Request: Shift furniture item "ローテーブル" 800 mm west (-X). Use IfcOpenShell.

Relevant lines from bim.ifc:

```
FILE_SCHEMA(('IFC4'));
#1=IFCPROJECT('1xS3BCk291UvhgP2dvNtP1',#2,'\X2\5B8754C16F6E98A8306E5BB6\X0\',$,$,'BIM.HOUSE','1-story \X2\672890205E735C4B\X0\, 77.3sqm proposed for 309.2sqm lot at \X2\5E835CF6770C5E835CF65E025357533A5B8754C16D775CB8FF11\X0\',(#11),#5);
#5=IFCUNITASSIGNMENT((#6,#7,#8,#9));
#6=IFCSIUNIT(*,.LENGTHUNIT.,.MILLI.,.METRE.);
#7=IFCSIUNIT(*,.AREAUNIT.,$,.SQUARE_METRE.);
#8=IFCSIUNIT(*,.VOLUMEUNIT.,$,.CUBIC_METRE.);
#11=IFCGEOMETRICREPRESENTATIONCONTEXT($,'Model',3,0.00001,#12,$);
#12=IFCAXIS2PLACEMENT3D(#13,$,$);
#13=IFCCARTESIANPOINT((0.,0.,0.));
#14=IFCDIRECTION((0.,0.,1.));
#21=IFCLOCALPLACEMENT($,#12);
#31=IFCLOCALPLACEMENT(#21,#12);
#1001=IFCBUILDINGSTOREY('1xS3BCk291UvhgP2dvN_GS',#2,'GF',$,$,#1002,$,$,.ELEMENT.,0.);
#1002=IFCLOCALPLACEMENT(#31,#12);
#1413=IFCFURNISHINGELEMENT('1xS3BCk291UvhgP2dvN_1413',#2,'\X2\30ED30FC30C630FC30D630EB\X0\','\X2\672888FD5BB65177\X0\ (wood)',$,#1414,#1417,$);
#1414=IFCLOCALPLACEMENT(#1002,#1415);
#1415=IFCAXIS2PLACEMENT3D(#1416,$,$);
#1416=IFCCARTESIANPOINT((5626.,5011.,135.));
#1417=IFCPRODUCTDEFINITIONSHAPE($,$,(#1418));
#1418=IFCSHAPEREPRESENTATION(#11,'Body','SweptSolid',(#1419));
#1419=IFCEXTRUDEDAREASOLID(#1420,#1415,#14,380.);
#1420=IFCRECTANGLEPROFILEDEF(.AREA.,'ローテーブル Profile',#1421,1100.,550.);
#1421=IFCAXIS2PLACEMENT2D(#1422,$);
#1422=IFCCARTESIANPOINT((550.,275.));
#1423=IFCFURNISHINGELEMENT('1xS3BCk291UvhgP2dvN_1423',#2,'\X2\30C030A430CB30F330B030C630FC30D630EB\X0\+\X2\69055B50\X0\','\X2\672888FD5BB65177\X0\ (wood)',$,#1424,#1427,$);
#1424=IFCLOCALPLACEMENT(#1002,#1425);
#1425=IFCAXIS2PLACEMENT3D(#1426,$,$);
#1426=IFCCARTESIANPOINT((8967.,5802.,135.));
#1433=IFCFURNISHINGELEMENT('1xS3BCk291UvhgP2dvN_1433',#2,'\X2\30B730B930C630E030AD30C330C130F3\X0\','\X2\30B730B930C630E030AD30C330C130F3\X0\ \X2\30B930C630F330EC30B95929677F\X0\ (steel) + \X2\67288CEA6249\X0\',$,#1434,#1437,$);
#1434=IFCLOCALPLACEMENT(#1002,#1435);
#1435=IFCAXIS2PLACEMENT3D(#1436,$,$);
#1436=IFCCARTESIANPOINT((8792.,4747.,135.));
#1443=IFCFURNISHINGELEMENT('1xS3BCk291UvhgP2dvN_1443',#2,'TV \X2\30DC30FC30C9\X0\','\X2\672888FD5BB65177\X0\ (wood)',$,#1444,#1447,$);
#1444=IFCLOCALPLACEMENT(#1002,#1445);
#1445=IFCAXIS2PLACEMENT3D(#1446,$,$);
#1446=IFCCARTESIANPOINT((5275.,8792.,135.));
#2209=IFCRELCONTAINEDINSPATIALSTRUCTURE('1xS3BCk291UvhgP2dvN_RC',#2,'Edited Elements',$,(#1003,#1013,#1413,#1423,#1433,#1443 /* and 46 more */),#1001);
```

```python
import ifcopenshell
import ifcopenshell.api.geometry
import ifcopenshell.util.placement
import ifcopenshell.util.unit

model = ifcopenshell.open("bim.ifc")
unit_scale = ifcopenshell.util.unit.calculate_unit_scale(model)

item = model.by_id(1413)
matrix = ifcopenshell.util.placement.get_local_placement(item.ObjectPlacement)
matrix[0, 3] -= 0.8 / unit_scale
ifcopenshell.api.geometry.edit_object_placement(model, product=item, matrix=matrix, is_si=False)

print(ifcopenshell.util.placement.get_local_placement(item.ObjectPlacement).round(3) + 0.0)

model.write("bim_updated.ifc")
```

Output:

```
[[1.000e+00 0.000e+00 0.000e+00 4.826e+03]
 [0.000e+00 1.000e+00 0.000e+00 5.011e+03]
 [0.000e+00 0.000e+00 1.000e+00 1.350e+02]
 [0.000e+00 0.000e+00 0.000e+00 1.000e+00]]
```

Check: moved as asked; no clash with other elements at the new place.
